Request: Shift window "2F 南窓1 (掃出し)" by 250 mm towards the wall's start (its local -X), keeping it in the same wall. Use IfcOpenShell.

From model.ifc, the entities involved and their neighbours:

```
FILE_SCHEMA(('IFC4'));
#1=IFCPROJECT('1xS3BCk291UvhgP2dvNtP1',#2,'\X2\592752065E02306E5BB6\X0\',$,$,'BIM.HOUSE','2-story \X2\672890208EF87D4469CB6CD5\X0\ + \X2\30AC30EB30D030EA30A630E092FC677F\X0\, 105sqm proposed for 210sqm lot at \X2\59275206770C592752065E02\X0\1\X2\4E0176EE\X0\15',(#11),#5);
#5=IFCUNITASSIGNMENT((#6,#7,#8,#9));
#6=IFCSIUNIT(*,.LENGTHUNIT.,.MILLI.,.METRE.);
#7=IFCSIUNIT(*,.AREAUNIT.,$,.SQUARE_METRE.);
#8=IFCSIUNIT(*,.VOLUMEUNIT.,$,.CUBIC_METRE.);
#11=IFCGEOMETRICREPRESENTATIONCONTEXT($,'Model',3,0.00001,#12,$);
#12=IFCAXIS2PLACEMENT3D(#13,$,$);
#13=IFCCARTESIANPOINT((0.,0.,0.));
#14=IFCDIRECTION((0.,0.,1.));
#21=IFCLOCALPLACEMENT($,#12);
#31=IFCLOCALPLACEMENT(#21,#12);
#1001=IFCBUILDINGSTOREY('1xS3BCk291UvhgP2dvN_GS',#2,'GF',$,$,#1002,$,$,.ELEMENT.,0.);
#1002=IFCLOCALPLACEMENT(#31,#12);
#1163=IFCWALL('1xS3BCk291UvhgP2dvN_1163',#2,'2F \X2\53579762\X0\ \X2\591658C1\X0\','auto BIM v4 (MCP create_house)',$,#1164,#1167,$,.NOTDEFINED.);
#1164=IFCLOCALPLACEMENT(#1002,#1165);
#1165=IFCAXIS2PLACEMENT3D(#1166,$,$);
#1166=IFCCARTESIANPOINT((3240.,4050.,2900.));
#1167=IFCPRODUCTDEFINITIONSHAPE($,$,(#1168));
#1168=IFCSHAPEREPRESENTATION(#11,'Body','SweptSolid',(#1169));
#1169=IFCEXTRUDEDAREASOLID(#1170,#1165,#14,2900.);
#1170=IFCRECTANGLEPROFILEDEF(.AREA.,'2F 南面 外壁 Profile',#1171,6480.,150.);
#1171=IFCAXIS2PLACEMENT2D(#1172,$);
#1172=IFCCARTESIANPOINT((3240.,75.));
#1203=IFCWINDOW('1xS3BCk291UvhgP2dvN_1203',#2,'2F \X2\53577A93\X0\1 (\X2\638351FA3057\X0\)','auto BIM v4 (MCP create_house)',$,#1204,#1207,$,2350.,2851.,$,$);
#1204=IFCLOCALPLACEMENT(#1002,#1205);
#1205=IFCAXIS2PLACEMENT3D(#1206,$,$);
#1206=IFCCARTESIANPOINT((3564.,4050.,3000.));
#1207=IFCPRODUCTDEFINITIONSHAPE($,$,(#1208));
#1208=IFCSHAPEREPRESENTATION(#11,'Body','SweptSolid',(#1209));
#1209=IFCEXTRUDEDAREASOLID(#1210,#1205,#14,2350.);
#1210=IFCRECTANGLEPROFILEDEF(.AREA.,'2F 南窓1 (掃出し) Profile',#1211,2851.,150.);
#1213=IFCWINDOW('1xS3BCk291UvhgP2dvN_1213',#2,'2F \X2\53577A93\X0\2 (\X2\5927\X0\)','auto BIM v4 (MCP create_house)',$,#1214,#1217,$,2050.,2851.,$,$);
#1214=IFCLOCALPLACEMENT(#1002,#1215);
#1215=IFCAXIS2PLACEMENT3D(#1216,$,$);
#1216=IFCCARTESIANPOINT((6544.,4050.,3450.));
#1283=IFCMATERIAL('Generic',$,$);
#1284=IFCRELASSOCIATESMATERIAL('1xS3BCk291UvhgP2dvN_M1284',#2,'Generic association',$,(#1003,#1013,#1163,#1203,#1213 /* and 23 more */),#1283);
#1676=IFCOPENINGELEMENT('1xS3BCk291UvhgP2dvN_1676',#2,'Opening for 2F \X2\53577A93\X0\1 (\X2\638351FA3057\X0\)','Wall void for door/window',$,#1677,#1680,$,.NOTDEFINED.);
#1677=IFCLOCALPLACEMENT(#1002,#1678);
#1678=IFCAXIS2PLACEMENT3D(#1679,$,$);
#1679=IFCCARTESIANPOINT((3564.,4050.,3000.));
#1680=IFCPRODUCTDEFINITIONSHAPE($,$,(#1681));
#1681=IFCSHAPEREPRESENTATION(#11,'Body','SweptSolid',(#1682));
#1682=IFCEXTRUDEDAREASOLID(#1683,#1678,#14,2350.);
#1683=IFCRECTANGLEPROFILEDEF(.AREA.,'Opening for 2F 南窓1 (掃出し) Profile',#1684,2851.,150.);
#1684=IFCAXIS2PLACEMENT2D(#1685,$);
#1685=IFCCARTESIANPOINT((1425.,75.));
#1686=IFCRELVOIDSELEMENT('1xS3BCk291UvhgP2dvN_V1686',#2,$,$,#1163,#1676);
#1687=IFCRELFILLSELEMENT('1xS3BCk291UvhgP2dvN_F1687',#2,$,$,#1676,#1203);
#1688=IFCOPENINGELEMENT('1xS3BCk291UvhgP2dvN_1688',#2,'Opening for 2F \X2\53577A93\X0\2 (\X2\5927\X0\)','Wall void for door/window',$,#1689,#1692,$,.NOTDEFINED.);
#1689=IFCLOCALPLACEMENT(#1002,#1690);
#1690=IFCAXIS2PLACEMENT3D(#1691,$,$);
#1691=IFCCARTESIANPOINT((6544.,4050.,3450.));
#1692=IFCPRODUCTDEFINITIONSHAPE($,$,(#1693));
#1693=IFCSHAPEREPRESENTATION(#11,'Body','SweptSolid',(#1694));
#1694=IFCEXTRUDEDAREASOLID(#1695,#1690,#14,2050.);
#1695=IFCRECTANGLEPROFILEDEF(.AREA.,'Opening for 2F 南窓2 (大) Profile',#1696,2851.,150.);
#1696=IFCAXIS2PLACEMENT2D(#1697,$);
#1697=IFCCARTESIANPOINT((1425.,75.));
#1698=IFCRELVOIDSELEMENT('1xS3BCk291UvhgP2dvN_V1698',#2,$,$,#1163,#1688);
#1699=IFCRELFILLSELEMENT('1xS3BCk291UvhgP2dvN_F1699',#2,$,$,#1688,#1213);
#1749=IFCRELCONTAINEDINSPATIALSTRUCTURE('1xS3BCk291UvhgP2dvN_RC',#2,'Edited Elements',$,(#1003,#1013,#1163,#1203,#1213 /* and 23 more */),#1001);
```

```python
import ifcopenshell
import ifcopenshell.api.geometry
import ifcopenshell.util.placement
import ifcopenshell.util.unit

model = ifcopenshell.open("model.ifc")
unit_scale = ifcopenshell.util.unit.calculate_unit_scale(model)

window = model.by_guid("1xS3BCk291UvhgP2dvN_1203")
opening = window.FillsVoids[0].RelatingOpeningElement
wall = opening.VoidsElements[0].RelatingBuildingElement

wall_matrix = ifcopenshell.util.placement.get_local_placement(wall.ObjectPlacement)
shift = wall_matrix[:3, 0] * -0.25 / unit_scale
before = ifcopenshell.util.placement.get_local_placement(window.ObjectPlacement)[:3, 3].copy()

# The window is not placed relative to its opening, so move both.
for product in (opening, window):
    matrix = ifcopenshell.util.placement.get_local_placement(product.ObjectPlacement)
    matrix[:3, 3] += shift
    ifcopenshell.api.geometry.edit_object_placement(model, product=product, matrix=matrix, is_si=False)

after = ifcopenshell.util.placement.get_local_placement(window.ObjectPlacement)[:3, 3]
print("window moved by", (after - before).round(3) + 0.0)

model.write("model_edited.ifc")
```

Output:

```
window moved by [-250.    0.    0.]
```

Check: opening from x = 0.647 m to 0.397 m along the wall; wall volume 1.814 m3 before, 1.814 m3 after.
